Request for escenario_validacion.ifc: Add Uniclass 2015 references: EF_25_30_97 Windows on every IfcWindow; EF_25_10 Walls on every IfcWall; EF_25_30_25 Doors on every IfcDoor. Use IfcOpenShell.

First a look at what the model holds.

```python
import ifcopenshell

model = ifcopenshell.open("escenario_validacion.ifc")
print(model.schema)
print("classifications:", [c.Name for c in model.by_type("IfcClassification")])
for ifc_class in ("IfcDoor", "IfcRoof", "IfcStair", "IfcWall", "IfcWindow"):
    print(ifc_class, len(model.by_type(ifc_class)))
```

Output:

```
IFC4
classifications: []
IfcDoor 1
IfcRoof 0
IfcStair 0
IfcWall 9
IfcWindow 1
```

```python
import ifcopenshell
import ifcopenshell.api.classification

model = ifcopenshell.open("escenario_validacion.ifc")

system = ifcopenshell.api.classification.add_classification(model, classification="Uniclass 2015")

codes = {
    "IfcWindow": ("EF_25_30_97", "Windows"),
    "IfcWall": ("EF_25_10", "Walls"),
    "IfcDoor": ("EF_25_30_25", "Doors"),
}
for ifc_class, (code, name) in codes.items():
    products = model.by_type(ifc_class)
    ifcopenshell.api.classification.add_reference(
        model, products=products, classification=system, identification=code, name=name
    )
    print(code, len(products))

model.write("escenario_validacion_edited.ifc")
```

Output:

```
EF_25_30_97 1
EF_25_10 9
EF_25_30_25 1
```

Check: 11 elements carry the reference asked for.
